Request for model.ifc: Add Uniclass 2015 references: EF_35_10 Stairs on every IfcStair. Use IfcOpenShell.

First a look at what the model holds.

```python
import ifcopenshell

model = ifcopenshell.open("model.ifc")
print(model.schema)
print("classifications:", [c.Name for c in model.by_type("IfcClassification")])
for ifc_class in ("IfcDoor", "IfcRoof", "IfcStair", "IfcWall", "IfcWindow"):
    print(ifc_class, len(model.by_type(ifc_class)))
```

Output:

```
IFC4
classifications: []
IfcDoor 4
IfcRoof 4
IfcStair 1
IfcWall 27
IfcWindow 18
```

```python
import ifcopenshell
import ifcopenshell.api.classification

model = ifcopenshell.open("model.ifc")

system = ifcopenshell.api.classification.add_classification(model, classification="Uniclass 2015")

codes = {
    "IfcStair": ("EF_35_10", "Stairs"),
}
for ifc_class, (code, name) in codes.items():
    products = model.by_type(ifc_class)
    ifcopenshell.api.classification.add_reference(
        model, products=products, classification=system, identification=code, name=name
    )
    print(code, len(products))

model.write("model_edited.ifc")
```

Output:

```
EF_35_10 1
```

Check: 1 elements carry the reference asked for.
